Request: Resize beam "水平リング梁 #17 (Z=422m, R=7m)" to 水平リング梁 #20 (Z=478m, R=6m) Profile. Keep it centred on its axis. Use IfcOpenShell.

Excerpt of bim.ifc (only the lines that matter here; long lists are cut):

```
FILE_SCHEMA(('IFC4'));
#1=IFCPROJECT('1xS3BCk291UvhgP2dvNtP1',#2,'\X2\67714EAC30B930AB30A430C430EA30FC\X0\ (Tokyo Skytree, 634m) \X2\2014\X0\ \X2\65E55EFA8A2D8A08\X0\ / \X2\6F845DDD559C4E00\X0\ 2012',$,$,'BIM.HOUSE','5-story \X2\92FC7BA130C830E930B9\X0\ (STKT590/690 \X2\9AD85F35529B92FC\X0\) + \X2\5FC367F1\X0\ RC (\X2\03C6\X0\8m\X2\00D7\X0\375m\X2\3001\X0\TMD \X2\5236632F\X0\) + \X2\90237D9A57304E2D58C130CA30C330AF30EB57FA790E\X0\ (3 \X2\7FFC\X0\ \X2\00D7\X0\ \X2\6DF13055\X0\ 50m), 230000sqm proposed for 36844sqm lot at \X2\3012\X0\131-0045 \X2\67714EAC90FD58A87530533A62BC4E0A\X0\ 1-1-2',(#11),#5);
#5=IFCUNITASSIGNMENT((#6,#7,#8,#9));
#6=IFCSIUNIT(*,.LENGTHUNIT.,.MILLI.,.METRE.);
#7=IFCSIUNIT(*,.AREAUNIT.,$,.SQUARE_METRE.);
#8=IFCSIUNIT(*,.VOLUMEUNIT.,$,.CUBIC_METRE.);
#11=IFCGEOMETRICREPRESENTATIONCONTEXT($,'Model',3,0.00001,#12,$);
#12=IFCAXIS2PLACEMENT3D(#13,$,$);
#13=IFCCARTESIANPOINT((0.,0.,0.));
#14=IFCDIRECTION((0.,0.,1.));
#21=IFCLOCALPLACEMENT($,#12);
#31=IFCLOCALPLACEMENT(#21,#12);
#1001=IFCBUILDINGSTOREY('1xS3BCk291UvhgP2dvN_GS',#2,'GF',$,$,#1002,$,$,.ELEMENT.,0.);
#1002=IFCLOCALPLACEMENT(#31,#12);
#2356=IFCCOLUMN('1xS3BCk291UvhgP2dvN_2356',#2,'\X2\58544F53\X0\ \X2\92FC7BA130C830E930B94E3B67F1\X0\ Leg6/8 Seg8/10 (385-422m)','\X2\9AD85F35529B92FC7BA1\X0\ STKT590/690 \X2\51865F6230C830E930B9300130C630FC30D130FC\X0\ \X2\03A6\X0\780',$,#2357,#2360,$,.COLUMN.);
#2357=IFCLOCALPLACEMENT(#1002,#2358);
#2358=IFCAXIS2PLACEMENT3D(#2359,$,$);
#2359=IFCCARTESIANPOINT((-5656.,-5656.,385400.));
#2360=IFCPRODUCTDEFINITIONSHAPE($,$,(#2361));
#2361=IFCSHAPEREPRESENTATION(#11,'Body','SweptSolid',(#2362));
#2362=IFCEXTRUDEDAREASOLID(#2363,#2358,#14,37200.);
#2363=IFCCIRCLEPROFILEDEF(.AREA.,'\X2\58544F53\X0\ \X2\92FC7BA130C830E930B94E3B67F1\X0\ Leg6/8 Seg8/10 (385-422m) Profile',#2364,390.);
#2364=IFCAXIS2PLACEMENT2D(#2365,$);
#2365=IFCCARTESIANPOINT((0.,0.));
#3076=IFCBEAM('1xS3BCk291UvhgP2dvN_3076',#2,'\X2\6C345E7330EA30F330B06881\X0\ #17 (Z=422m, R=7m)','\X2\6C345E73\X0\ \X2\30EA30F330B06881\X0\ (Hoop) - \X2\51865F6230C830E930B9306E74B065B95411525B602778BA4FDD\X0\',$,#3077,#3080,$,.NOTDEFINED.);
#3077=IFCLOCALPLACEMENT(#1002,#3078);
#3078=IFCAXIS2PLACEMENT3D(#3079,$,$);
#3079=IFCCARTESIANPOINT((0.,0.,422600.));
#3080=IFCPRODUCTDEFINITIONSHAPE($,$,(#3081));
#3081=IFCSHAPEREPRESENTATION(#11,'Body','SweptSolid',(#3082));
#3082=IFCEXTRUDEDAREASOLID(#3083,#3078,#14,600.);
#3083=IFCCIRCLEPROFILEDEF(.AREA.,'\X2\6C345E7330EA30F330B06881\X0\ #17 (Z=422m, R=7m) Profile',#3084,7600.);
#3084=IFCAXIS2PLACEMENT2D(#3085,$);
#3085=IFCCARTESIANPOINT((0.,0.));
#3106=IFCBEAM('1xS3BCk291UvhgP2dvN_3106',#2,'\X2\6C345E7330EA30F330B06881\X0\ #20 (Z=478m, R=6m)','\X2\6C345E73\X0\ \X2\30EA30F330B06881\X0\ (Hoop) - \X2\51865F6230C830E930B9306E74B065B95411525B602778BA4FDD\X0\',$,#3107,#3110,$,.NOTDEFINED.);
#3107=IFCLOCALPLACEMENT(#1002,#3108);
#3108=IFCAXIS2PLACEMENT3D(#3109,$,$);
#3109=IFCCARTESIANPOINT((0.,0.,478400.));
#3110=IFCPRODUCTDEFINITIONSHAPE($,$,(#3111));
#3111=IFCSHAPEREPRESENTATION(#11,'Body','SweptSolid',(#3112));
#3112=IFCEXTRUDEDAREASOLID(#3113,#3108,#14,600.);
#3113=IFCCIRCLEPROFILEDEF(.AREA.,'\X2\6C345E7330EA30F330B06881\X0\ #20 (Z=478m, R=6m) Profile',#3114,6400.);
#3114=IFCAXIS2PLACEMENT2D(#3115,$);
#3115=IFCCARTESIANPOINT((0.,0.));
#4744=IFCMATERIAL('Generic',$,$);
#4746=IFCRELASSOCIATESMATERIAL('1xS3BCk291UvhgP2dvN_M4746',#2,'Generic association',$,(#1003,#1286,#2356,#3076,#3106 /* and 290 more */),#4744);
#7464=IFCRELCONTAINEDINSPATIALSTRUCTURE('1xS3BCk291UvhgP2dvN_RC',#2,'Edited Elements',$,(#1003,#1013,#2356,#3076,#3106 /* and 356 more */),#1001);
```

```python
import ifcopenshell
import ifcopenshell.util.element

model = ifcopenshell.open("bim.ifc")

member = model.by_guid("1xS3BCk291UvhgP2dvN_3076")
source = next(p for p in model.by_type("IfcCircleProfileDef") if p.ProfileName == "水平リング梁 #20 (Z=478m, R=6m) Profile")

body = next(r for r in member.Representation.Representations if r.RepresentationIdentifier == "Body")
solid = body.Items[0]
old_profile = solid.SweptArea

# Copy the section's sizes but keep this member's own profile position.
profile = ifcopenshell.util.element.copy(model, source)
profile.Position = old_profile.Position
solid.SweptArea = profile
if not model.get_total_inverses(old_profile):
    ifcopenshell.util.element.remove_deep2(model, old_profile)

print(solid.SweptArea)

model.write("bim_updated.ifc")
```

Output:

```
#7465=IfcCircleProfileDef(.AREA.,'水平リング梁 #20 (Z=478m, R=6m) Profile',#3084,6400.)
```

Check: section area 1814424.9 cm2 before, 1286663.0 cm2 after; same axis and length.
